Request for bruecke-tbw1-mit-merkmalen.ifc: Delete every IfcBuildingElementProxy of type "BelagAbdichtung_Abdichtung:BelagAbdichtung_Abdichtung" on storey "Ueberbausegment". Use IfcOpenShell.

First a look at what the model holds.

```python
import ifcopenshell
import ifcopenshell.util.element

model = ifcopenshell.open("bruecke-tbw1-mit-merkmalen.ifc")
print(model.schema)
storey = next(s for s in model.by_type("IfcBuildingStorey") if s.Name == "Ueberbausegment")
proxies = [e for e in ifcopenshell.util.element.get_decomposition(storey) if e.is_a("IfcBuildingElementProxy")]
seen = {}
for e in proxies:
    element_type = ifcopenshell.util.element.get_type(e)
    name = element_type.Name if element_type not in (None, e) else None
    seen[name] = seen.get(name, 0) + 1
for name, count in sorted(seen.items(), key=str):
    print(count, "x", name)
```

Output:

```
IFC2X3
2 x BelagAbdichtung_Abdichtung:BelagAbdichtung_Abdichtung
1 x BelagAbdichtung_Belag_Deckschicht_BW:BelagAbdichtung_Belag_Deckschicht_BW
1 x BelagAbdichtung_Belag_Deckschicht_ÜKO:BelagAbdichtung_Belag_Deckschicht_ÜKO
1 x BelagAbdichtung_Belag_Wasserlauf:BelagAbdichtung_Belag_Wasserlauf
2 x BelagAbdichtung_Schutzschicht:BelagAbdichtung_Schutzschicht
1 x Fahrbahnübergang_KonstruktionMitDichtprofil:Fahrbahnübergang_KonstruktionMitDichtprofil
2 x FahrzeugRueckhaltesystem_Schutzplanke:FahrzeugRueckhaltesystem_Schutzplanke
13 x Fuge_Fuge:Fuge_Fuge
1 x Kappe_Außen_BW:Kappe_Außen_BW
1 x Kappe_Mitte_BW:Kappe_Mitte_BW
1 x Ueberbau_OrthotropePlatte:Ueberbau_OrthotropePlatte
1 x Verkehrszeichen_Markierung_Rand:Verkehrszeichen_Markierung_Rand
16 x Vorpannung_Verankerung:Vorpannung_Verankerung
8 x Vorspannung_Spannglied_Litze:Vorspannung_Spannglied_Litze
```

```python
import ifcopenshell
import ifcopenshell.api.root
import ifcopenshell.util.element

model = ifcopenshell.open("bruecke-tbw1-mit-merkmalen.ifc")

storey = next(s for s in model.by_type("IfcBuildingStorey") if s.Name == "Ueberbausegment")
proxies = [e for e in ifcopenshell.util.element.get_decomposition(storey) if e.is_a("IfcBuildingElementProxy")]
targets = [e for e in proxies if (t := ifcopenshell.util.element.get_type(e)) not in (None, e) and t.Name == "BelagAbdichtung_Abdichtung:BelagAbdichtung_Abdichtung"]

for e in targets:
    ifcopenshell.api.root.remove_product(model, product=e)
print(len(targets), "removed")

model.write("bruecke-tbw1-mit-merkmalen_v2.ifc")
```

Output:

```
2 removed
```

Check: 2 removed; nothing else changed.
